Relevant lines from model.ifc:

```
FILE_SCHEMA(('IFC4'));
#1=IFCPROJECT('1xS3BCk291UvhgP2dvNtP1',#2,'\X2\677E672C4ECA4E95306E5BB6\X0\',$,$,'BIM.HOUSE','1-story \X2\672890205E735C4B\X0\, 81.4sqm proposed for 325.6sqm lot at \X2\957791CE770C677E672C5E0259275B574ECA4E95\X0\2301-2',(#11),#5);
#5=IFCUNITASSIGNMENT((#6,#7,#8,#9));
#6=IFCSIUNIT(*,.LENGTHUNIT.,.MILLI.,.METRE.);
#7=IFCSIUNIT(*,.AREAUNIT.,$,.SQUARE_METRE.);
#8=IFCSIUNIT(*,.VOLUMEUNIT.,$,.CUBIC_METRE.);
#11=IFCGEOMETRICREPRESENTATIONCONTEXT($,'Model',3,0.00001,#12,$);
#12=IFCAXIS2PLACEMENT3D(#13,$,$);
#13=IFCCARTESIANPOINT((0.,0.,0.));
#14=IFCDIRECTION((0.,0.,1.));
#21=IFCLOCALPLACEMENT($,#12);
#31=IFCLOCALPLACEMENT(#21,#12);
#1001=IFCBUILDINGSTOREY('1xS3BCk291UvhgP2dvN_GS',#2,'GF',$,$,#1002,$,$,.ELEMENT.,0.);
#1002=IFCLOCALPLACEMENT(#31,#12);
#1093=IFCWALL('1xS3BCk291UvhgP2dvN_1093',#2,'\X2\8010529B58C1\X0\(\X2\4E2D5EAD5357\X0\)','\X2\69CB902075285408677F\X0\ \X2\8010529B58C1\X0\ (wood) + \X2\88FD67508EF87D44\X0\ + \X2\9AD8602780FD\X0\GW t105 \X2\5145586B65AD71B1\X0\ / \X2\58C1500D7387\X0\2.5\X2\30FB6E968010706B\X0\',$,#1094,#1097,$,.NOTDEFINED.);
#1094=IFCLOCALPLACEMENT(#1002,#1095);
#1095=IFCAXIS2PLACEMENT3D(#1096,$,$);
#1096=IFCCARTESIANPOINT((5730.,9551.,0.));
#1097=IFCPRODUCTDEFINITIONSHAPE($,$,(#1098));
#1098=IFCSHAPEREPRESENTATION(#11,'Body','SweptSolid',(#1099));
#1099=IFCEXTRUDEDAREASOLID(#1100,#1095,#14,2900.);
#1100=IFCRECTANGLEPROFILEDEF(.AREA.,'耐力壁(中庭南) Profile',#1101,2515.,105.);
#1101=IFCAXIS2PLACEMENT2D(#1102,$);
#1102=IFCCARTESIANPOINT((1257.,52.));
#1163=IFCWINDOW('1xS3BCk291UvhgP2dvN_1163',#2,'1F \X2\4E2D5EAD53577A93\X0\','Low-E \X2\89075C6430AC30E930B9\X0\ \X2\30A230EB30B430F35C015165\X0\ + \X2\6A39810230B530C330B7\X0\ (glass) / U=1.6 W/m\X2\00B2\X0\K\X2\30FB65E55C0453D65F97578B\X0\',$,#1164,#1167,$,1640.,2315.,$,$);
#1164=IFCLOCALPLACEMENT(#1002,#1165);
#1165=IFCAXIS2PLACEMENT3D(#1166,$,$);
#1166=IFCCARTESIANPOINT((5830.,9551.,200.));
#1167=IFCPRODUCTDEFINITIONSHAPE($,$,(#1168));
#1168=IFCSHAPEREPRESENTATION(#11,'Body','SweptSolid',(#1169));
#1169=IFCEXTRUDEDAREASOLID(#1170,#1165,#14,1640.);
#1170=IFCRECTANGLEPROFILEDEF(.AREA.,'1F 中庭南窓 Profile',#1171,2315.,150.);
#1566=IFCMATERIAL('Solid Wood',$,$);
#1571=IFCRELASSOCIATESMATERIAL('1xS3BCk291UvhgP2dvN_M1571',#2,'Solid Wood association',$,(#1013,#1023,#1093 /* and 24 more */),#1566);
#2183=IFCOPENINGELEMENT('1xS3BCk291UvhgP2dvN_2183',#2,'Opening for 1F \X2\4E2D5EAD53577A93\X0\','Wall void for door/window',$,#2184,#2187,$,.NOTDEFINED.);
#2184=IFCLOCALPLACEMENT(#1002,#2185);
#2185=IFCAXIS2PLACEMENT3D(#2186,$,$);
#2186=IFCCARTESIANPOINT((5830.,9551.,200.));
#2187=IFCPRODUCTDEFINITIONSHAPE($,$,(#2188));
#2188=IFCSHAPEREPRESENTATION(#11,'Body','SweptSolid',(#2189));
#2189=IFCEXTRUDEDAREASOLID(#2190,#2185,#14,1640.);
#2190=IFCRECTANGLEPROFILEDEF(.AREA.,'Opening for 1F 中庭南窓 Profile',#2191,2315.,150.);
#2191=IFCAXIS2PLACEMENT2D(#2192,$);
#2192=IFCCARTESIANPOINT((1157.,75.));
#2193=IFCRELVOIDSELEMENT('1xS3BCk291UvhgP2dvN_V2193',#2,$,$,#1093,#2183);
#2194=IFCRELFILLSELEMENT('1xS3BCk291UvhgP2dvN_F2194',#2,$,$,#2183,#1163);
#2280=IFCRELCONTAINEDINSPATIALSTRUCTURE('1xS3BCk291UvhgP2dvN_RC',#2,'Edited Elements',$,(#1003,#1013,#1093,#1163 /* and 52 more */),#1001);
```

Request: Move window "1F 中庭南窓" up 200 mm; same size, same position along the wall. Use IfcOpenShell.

```python
import numpy as np
import ifcopenshell
import ifcopenshell.api.geometry
import ifcopenshell.util.placement
import ifcopenshell.util.unit

model = ifcopenshell.open("model.ifc")
unit_scale = ifcopenshell.util.unit.calculate_unit_scale(model)

window = model.by_id(1163)
opening = window.FillsVoids[0].RelatingOpeningElement
dz = 0.2 / unit_scale

shift = np.array([0.0, 0.0, dz])
# The window is not placed relative to its opening, so move both.
for product in (opening, window):
    matrix = ifcopenshell.util.placement.get_local_placement(product.ObjectPlacement)
    matrix[:3, 3] += shift
    ifcopenshell.api.geometry.edit_object_placement(model, product=product, matrix=matrix, is_si=False)

print(f"moved by {dz * unit_scale:+.3f} m")

model.write("model-out.ifc")
```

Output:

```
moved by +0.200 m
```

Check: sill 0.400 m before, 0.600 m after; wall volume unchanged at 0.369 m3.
